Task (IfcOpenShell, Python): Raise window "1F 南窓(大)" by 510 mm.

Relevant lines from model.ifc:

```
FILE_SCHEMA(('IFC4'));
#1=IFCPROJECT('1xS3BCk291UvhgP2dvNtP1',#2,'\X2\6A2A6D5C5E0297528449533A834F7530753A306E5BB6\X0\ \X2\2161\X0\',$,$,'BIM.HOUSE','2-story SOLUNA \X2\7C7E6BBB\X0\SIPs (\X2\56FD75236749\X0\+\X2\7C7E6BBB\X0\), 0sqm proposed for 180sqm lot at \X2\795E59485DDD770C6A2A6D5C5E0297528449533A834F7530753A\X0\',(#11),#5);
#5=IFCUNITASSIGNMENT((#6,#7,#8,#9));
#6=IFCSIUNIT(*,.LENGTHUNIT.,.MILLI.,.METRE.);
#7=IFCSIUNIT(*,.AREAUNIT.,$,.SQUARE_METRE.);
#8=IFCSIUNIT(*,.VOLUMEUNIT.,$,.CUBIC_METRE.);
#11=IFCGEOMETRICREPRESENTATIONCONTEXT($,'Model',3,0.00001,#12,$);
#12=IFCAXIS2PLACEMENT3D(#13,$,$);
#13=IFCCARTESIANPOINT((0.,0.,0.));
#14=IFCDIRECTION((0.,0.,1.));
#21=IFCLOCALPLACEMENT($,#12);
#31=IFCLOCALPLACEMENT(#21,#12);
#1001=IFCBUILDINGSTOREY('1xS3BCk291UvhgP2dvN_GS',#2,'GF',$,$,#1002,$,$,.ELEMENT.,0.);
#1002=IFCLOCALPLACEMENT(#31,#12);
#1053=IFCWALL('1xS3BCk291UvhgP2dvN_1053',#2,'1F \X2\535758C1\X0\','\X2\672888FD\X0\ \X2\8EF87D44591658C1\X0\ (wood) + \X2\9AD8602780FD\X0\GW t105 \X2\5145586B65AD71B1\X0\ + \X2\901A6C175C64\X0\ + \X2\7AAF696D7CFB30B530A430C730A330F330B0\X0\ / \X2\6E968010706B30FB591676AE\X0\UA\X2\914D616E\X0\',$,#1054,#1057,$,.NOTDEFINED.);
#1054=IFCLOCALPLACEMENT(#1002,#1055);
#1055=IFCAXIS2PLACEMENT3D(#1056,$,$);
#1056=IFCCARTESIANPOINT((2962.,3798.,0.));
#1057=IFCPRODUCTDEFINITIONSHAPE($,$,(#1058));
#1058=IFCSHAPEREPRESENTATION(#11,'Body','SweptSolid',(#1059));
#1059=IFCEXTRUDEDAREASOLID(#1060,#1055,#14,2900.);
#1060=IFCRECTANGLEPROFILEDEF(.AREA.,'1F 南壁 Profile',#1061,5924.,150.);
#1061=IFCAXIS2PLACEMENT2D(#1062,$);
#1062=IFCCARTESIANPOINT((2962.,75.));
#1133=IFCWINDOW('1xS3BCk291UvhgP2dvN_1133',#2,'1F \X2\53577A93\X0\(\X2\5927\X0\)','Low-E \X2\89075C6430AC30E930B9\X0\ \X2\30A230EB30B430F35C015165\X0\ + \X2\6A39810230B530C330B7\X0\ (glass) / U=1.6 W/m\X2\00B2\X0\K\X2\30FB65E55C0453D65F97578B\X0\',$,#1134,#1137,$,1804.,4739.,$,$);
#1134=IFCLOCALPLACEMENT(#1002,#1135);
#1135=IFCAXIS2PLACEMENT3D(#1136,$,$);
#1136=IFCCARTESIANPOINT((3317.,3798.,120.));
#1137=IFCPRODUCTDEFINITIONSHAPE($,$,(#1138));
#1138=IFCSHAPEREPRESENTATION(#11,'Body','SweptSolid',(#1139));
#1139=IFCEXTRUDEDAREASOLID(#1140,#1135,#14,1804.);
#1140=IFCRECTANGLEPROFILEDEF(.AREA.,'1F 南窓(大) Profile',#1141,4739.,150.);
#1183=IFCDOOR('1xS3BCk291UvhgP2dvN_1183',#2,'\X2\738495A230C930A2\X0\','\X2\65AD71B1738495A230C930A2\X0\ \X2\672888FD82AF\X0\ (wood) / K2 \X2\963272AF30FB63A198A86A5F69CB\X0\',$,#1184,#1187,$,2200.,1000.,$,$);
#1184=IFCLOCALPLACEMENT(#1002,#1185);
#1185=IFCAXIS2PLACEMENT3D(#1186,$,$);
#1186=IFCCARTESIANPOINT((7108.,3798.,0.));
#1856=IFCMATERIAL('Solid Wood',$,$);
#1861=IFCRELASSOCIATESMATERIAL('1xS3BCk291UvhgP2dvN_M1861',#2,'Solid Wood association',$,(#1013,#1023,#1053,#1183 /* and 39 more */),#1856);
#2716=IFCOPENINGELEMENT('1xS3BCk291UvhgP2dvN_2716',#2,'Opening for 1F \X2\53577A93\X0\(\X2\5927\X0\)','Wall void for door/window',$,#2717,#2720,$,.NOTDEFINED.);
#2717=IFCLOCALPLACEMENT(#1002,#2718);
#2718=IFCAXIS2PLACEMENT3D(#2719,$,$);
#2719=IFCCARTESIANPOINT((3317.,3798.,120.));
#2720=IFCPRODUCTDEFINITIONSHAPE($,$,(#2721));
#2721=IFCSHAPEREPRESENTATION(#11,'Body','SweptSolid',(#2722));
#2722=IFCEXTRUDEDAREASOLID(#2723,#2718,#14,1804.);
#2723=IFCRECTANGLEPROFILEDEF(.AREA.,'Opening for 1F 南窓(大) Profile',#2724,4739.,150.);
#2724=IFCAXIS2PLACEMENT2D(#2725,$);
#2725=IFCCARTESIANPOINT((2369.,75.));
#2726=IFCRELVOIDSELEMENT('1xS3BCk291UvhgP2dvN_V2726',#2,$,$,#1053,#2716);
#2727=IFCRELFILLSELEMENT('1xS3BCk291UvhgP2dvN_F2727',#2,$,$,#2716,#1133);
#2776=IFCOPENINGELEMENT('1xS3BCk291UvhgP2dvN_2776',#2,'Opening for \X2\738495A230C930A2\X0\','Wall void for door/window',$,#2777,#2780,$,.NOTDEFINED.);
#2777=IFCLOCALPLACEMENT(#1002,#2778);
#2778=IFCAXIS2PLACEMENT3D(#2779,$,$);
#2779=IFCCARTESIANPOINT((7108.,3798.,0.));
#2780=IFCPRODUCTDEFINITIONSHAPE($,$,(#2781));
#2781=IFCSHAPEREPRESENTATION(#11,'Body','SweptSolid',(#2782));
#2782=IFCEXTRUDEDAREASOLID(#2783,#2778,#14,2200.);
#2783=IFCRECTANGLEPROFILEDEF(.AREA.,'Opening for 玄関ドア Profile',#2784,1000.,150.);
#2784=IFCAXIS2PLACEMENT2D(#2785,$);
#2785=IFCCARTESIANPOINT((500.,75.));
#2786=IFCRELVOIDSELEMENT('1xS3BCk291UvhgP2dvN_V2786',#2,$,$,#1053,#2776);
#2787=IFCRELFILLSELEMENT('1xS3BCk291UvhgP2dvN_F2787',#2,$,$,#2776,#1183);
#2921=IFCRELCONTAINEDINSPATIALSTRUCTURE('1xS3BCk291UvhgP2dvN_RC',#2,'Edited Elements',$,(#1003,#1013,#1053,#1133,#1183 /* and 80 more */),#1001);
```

```python
import numpy as np
import ifcopenshell
import ifcopenshell.api.geometry
import ifcopenshell.util.placement
import ifcopenshell.util.unit

model = ifcopenshell.open("model.ifc")
unit_scale = ifcopenshell.util.unit.calculate_unit_scale(model)

window = model.by_id(1133)
opening = window.FillsVoids[0].RelatingOpeningElement
dz = 0.51 / unit_scale

shift = np.array([0.0, 0.0, dz])
# The window is not placed relative to its opening, so move both.
for product in (opening, window):
    matrix = ifcopenshell.util.placement.get_local_placement(product.ObjectPlacement)
    matrix[:3, 3] += shift
    ifcopenshell.api.geometry.edit_object_placement(model, product=product, matrix=matrix, is_si=False)

print(f"moved by {dz * unit_scale:+.3f} m")

model.write("model-out.ifc")
```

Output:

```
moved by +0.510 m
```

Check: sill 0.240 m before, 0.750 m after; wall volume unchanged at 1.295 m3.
